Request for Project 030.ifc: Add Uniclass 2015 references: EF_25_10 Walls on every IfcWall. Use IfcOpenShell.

First a look at what the model holds.

```python
import ifcopenshell

model = ifcopenshell.open("Project 030.ifc")
print(model.schema)
print("classifications:", [c.Name for c in model.by_type("IfcClassification")])
for ifc_class in ("IfcDoor", "IfcRoof", "IfcStair", "IfcWall", "IfcWindow"):
    print(ifc_class, len(model.by_type(ifc_class)))
```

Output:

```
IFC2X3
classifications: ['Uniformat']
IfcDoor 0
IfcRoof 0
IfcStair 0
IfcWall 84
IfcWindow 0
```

```python
import ifcopenshell
import ifcopenshell.api.classification

model = ifcopenshell.open("Project 030.ifc")

# IFC2X3 requires Source and Edition and has no link from the project to the system.
system = model.create_entity("IfcClassification", Source="NBS", Edition="2015", Name="Uniclass 2015")

codes = {
    "IfcWall": ("EF_25_10", "Walls"),
}
for ifc_class, (code, name) in codes.items():
    products = model.by_type(ifc_class)
    ifcopenshell.api.classification.add_reference(
        model, products=products, classification=system, identification=code, name=name
    )
    print(code, len(products))

model.write("Project 030_rev.ifc")
```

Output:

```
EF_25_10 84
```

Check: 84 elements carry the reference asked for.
